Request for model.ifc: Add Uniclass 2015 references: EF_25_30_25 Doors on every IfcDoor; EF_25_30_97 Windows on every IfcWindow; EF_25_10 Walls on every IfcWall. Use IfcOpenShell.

First a look at what the model holds.

```python
import ifcopenshell

model = ifcopenshell.open("model.ifc")
print(model.schema)
print("classifications:", [c.Name for c in model.by_type("IfcClassification")])
for ifc_class in ("IfcDoor", "IfcRoof", "IfcStair", "IfcWall", "IfcWindow"):
    print(ifc_class, len(model.by_type(ifc_class)))
```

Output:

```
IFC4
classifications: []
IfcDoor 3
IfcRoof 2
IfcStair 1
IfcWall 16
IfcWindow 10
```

```python
import ifcopenshell
import ifcopenshell.api.classification

model = ifcopenshell.open("model.ifc")

system = ifcopenshell.api.classification.add_classification(model, classification="Uniclass 2015")

codes = {
    "IfcDoor": ("EF_25_30_25", "Doors"),
    "IfcWindow": ("EF_25_30_97", "Windows"),
    "IfcWall": ("EF_25_10", "Walls"),
}
for ifc_class, (code, name) in codes.items():
    products = model.by_type(ifc_class)
    ifcopenshell.api.classification.add_reference(
        model, products=products, classification=system, identification=code, name=name
    )
    print(code, len(products))

model.write("model-out.ifc")
```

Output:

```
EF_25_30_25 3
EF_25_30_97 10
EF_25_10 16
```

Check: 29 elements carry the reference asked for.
